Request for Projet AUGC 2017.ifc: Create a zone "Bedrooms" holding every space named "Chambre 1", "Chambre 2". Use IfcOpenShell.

First a look at what the model holds.

```python
import ifcopenshell

model = ifcopenshell.open("Projet AUGC 2017.ifc")
print(model.schema)
seen = {}
for space in model.by_type("IfcSpace"):
    seen[space.LongName] = seen.get(space.LongName, 0) + 1
for name, count in sorted(seen.items(), key=str):
    print(count, "x", name)
print("zones:", [z.Name for z in model.by_type("IfcZone")][:20])
```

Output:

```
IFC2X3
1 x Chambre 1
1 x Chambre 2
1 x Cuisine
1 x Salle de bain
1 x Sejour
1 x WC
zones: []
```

```python
import ifcopenshell
import ifcopenshell.api.group
import ifcopenshell.api.root

model = ifcopenshell.open("Projet AUGC 2017.ifc")

names = {"Chambre 1", "Chambre 2"}
spaces = [s for s in model.by_type("IfcSpace") if s.LongName in names]

zone = ifcopenshell.api.root.create_entity(model, ifc_class="IfcZone", name="Bedrooms")
ifcopenshell.api.group.assign_group(model, products=spaces, group=zone)
print(len(spaces), "spaces in", zone.Name)

model.write("Projet AUGC 2017-out.ifc")
```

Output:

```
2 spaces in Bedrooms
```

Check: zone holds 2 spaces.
